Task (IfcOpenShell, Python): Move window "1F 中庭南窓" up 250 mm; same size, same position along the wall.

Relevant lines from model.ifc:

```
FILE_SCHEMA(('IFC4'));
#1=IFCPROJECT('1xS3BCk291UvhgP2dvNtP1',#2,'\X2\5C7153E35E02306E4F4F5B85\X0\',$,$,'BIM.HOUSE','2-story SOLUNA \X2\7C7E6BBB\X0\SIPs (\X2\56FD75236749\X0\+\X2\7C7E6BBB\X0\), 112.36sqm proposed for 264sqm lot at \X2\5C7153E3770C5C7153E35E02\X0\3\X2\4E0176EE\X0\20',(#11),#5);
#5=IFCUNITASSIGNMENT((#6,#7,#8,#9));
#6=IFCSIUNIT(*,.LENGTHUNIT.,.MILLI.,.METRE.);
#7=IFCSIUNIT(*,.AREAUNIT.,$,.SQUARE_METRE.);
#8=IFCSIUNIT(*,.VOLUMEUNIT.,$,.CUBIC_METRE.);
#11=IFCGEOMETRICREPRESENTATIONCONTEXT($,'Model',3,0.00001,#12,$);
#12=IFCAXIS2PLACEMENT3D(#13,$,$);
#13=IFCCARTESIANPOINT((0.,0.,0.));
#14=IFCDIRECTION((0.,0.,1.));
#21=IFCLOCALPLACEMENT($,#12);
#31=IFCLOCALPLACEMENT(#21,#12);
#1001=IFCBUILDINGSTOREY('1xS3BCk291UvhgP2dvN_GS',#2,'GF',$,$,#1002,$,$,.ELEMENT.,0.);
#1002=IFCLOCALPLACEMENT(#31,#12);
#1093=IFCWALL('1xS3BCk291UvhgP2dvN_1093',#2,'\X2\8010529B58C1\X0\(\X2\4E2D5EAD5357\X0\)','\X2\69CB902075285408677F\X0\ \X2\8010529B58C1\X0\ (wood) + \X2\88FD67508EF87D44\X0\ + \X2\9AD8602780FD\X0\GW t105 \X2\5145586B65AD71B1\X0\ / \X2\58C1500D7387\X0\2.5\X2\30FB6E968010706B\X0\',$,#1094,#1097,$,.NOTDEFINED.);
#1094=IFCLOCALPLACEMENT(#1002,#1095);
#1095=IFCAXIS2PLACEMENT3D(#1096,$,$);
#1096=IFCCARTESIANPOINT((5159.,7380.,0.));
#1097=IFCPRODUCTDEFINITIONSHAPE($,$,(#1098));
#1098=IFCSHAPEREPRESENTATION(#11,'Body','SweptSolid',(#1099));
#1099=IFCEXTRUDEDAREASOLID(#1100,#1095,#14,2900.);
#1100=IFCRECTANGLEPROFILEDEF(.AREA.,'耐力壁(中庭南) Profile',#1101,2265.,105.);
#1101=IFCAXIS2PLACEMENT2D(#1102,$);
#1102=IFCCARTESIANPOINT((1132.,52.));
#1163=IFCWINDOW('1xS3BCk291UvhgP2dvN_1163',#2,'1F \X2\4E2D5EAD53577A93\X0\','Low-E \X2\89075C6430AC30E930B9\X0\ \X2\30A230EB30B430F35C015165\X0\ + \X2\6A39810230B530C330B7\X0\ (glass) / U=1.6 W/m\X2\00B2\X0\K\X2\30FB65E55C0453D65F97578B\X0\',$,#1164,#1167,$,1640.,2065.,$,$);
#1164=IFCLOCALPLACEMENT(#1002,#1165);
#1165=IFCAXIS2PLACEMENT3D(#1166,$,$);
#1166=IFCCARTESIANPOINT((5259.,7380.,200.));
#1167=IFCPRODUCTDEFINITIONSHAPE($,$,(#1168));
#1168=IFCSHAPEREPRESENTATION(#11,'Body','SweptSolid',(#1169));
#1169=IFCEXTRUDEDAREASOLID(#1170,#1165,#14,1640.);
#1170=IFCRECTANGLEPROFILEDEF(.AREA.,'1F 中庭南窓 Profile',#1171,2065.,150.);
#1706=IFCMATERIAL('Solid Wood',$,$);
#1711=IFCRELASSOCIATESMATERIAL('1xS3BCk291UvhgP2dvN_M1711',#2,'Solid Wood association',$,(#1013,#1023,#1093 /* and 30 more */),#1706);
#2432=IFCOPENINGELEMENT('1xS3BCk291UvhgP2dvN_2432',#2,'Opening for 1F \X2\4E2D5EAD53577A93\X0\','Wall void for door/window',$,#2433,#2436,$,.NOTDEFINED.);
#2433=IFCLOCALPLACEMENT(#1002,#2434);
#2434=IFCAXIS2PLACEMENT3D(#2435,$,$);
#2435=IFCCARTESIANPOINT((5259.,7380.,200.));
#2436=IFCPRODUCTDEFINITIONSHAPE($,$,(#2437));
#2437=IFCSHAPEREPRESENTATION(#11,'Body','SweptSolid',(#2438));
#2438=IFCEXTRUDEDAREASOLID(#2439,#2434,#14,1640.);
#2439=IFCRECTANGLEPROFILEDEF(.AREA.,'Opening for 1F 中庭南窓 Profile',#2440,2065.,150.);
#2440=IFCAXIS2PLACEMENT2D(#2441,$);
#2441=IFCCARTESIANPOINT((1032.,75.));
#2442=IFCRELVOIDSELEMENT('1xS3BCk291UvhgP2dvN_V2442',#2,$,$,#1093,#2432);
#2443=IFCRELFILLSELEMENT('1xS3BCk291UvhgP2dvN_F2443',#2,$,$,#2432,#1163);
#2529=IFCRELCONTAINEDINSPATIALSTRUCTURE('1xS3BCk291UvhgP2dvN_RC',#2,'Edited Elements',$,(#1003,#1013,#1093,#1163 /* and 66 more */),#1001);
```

```python
import numpy as np
import ifcopenshell
import ifcopenshell.api.geometry
import ifcopenshell.util.placement
import ifcopenshell.util.unit

model = ifcopenshell.open("model.ifc")
unit_scale = ifcopenshell.util.unit.calculate_unit_scale(model)

window = model.by_id(1163)
opening = window.FillsVoids[0].RelatingOpeningElement
dz = 0.25 / unit_scale

shift = np.array([0.0, 0.0, dz])
# The window is not placed relative to its opening, so move both.
for product in (opening, window):
    matrix = ifcopenshell.util.placement.get_local_placement(product.ObjectPlacement)
    matrix[:3, 3] += shift
    ifcopenshell.api.geometry.edit_object_placement(model, product=product, matrix=matrix, is_si=False)

print(f"moved by {dz * unit_scale:+.3f} m")

model.write("model_updated.ifc")
```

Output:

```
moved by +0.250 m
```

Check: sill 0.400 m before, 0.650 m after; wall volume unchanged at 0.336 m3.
